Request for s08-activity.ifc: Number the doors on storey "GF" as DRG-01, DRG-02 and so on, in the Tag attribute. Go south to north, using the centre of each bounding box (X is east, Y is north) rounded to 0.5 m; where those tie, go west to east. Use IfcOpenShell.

First a look at what the model holds.

```python
import ifcopenshell
import ifcopenshell.util.element
import ifcopenshell.util.placement

model = ifcopenshell.open("s08-activity.ifc")
print(model.schema)
storey = next(s for s in model.by_type("IfcBuildingStorey") if s.Name == "GF")
doors = [e for e in ifcopenshell.util.element.get_decomposition(storey) if e.is_a("IfcDoor")]
for e in sorted(doors, key=lambda e: e.id()):
    origin = ifcopenshell.util.placement.get_local_placement(e.ObjectPlacement)[:3, 3]
    print(e.id(), e.Tag, e.Name, origin.round(2) + 0.0, sep=" | ")
```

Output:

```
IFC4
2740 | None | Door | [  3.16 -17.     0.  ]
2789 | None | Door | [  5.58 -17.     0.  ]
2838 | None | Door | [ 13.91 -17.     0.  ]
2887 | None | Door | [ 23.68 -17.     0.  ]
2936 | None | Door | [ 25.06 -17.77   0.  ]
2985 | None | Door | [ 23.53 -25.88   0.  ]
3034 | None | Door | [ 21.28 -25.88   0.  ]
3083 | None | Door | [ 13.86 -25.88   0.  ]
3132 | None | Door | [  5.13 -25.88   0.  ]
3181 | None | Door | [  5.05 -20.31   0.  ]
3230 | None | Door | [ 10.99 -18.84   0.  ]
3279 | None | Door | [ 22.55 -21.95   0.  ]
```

```python
import ifcopenshell
import ifcopenshell.geom
import ifcopenshell.util.element
import ifcopenshell.util.shape

model = ifcopenshell.open("s08-activity.ifc")
settings = ifcopenshell.geom.settings()
settings.set("use-world-coords", True)


def centre(element):
    shape = ifcopenshell.geom.create_shape(settings, element)
    return ifcopenshell.util.shape.get_bbox_centroid(shape.geometry)


storey = next(s for s in model.by_type("IfcBuildingStorey") if s.Name == "GF")
doors = [e for e in ifcopenshell.util.element.get_decomposition(storey) if e.is_a("IfcDoor")]

# Insertion points can sit at a corner or the storey origin, so sort by the geometry (in metres).
centres = {e: centre(e) for e in doors}
doors.sort(key=lambda e: (round(centres[e][1] / 0.5), centres[e][0]))

for i, e in enumerate(doors, start=1):
    number = f"DRG-{i:02d}"
    e.Tag = number
    print(e.id(), number)

model.write("s08-activity_updated.ifc")
```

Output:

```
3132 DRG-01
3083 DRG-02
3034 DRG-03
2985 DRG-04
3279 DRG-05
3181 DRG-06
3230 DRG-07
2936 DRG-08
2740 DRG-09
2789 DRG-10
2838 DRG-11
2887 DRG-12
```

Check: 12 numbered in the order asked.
